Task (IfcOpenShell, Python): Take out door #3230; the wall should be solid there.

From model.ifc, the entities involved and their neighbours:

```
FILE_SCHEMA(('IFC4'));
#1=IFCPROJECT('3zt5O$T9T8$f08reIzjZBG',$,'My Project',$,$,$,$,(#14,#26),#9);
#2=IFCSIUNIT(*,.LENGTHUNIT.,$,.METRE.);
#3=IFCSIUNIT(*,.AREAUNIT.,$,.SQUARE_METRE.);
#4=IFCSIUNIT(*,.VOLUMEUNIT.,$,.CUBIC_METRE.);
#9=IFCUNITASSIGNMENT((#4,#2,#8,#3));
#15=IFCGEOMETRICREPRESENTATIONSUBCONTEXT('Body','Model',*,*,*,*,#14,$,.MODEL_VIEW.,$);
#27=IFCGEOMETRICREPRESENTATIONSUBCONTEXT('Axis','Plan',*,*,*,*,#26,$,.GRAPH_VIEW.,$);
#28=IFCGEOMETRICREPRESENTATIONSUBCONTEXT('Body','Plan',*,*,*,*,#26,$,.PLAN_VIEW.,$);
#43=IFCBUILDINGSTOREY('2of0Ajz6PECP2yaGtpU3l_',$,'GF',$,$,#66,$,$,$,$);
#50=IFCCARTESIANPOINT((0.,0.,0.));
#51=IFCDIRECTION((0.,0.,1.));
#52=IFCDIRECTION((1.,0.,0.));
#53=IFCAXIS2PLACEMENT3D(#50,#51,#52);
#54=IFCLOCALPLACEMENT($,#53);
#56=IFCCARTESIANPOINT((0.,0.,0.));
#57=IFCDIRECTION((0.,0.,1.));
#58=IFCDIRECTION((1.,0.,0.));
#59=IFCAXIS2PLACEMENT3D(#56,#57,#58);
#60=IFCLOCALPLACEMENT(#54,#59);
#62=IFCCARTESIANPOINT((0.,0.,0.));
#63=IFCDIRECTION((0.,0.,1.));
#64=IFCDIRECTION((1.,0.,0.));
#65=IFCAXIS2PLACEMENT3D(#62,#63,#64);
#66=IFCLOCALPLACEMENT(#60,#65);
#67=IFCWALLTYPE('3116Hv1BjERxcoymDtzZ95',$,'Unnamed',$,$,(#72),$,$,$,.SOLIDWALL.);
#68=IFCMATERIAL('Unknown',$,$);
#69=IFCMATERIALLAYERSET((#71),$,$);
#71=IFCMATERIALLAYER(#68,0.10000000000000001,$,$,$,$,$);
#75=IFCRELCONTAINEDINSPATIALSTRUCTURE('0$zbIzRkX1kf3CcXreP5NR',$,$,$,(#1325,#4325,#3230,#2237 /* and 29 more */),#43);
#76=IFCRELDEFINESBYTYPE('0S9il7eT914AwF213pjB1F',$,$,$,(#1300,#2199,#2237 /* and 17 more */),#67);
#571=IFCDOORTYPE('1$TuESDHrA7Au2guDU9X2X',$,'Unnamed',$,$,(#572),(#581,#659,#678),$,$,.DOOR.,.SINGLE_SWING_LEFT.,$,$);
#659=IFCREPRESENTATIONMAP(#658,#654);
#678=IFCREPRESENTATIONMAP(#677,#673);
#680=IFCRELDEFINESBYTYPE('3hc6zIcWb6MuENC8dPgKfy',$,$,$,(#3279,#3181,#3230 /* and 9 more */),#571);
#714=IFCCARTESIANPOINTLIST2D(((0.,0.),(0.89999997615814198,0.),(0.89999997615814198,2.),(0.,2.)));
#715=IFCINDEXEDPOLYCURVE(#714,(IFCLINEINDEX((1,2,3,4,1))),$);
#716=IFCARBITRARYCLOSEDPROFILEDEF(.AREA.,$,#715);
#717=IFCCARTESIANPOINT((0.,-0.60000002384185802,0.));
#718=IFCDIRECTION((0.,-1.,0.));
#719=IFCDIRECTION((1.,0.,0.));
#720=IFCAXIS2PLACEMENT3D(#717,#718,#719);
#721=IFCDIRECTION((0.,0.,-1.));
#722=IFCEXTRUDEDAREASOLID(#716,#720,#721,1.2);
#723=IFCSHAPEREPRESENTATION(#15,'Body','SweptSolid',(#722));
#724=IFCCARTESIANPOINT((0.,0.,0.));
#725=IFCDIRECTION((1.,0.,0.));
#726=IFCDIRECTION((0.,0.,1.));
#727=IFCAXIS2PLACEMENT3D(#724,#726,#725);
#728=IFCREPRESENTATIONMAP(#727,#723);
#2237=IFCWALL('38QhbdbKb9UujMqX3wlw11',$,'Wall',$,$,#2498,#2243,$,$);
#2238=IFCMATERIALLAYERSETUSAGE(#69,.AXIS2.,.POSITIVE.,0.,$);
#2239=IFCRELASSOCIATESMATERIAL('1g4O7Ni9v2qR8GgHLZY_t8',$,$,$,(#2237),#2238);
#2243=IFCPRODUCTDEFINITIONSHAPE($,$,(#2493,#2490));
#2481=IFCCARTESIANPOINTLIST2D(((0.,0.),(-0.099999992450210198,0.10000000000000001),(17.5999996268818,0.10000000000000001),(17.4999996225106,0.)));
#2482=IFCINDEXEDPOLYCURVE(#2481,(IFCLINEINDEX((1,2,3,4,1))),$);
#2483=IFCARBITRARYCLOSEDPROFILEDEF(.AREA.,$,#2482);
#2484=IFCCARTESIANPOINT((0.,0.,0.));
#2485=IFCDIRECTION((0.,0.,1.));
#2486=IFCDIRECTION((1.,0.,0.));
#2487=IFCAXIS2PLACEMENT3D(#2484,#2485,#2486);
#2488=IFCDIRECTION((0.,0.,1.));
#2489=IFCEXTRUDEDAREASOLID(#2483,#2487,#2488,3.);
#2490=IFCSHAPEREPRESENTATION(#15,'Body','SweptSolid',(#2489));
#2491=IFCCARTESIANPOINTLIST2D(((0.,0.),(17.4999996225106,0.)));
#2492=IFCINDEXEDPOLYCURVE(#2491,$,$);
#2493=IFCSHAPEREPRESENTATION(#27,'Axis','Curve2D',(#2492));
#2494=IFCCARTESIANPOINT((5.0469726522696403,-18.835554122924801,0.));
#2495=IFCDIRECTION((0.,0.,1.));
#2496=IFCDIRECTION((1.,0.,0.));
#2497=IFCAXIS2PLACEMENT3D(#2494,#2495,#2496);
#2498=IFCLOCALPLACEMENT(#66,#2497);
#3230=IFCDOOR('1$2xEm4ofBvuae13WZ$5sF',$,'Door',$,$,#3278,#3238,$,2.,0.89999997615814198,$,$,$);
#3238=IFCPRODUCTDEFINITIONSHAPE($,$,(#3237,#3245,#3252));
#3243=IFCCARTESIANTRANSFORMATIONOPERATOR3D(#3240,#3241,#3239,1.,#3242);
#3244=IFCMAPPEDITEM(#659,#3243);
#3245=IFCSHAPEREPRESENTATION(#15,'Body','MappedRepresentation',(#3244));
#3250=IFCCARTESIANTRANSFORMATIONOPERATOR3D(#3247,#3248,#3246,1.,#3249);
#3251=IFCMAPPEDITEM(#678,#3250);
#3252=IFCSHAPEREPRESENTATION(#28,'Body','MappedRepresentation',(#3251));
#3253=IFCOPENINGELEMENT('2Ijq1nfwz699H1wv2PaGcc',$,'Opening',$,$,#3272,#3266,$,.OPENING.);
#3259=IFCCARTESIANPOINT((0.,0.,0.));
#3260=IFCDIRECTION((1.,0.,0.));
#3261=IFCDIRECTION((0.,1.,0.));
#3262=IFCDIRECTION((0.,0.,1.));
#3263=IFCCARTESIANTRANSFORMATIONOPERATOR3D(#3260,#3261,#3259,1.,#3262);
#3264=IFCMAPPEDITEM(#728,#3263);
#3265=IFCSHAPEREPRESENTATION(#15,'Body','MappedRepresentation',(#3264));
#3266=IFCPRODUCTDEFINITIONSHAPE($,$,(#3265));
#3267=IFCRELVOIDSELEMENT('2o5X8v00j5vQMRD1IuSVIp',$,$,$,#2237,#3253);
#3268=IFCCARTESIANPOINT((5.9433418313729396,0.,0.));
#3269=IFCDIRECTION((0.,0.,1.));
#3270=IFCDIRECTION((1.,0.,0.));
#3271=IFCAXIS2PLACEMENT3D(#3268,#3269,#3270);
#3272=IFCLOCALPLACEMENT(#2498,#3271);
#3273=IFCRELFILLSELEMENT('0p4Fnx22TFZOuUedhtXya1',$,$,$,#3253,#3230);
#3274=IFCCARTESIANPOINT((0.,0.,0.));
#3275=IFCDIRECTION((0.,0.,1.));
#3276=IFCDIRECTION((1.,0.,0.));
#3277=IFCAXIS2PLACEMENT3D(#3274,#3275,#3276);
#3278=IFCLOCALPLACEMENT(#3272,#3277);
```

```python
import ifcopenshell
import ifcopenshell.api.feature
import ifcopenshell.api.root
import ifcopenshell.geom
import ifcopenshell.util.shape

model = ifcopenshell.open("model.ifc")
settings = ifcopenshell.geom.settings()


def volume(element):
    """Net volume in cubic metres, openings subtracted."""
    shape = ifcopenshell.geom.create_shape(settings, element)
    return ifcopenshell.util.shape.get_volume(shape.geometry)


door = model.by_guid("1$2xEm4ofBvuae13WZ$5sF")
opening = door.FillsVoids[0].RelatingOpeningElement
wall = opening.VoidsElements[0].RelatingBuildingElement
before = volume(wall)

ifcopenshell.api.root.remove_product(model, product=door)
ifcopenshell.api.feature.remove_feature(model, feature=opening)

after = volume(wall)

print(f"wall volume {before:.3f} -> {after:.3f} m3")

model.write("model_v2.ifc")
```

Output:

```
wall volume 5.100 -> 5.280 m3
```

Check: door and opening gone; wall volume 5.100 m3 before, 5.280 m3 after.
